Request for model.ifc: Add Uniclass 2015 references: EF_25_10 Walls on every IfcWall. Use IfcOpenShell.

First a look at what the model holds.

```python
import ifcopenshell

model = ifcopenshell.open("model.ifc")
print(model.schema)
print("classifications:", [c.Name for c in model.by_type("IfcClassification")])
for ifc_class in ("IfcDoor", "IfcRoof", "IfcStair", "IfcWall", "IfcWindow"):
    print(ifc_class, len(model.by_type(ifc_class)))
```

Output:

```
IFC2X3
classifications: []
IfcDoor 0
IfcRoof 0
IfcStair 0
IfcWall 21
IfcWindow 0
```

```python
import ifcopenshell
import ifcopenshell.api.classification

model = ifcopenshell.open("model.ifc")

# IFC2X3 requires Source and Edition and has no link from the project to the system.
system = model.create_entity("IfcClassification", Source="NBS", Edition="2015", Name="Uniclass 2015")

codes = {
    "IfcWall": ("EF_25_10", "Walls"),
}
for ifc_class, (code, name) in codes.items():
    products = model.by_type(ifc_class)
    ifcopenshell.api.classification.add_reference(
        model, products=products, classification=system, identification=code, name=name
    )
    print(code, len(products))

model.write("model-out.ifc")
```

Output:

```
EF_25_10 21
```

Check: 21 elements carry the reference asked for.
